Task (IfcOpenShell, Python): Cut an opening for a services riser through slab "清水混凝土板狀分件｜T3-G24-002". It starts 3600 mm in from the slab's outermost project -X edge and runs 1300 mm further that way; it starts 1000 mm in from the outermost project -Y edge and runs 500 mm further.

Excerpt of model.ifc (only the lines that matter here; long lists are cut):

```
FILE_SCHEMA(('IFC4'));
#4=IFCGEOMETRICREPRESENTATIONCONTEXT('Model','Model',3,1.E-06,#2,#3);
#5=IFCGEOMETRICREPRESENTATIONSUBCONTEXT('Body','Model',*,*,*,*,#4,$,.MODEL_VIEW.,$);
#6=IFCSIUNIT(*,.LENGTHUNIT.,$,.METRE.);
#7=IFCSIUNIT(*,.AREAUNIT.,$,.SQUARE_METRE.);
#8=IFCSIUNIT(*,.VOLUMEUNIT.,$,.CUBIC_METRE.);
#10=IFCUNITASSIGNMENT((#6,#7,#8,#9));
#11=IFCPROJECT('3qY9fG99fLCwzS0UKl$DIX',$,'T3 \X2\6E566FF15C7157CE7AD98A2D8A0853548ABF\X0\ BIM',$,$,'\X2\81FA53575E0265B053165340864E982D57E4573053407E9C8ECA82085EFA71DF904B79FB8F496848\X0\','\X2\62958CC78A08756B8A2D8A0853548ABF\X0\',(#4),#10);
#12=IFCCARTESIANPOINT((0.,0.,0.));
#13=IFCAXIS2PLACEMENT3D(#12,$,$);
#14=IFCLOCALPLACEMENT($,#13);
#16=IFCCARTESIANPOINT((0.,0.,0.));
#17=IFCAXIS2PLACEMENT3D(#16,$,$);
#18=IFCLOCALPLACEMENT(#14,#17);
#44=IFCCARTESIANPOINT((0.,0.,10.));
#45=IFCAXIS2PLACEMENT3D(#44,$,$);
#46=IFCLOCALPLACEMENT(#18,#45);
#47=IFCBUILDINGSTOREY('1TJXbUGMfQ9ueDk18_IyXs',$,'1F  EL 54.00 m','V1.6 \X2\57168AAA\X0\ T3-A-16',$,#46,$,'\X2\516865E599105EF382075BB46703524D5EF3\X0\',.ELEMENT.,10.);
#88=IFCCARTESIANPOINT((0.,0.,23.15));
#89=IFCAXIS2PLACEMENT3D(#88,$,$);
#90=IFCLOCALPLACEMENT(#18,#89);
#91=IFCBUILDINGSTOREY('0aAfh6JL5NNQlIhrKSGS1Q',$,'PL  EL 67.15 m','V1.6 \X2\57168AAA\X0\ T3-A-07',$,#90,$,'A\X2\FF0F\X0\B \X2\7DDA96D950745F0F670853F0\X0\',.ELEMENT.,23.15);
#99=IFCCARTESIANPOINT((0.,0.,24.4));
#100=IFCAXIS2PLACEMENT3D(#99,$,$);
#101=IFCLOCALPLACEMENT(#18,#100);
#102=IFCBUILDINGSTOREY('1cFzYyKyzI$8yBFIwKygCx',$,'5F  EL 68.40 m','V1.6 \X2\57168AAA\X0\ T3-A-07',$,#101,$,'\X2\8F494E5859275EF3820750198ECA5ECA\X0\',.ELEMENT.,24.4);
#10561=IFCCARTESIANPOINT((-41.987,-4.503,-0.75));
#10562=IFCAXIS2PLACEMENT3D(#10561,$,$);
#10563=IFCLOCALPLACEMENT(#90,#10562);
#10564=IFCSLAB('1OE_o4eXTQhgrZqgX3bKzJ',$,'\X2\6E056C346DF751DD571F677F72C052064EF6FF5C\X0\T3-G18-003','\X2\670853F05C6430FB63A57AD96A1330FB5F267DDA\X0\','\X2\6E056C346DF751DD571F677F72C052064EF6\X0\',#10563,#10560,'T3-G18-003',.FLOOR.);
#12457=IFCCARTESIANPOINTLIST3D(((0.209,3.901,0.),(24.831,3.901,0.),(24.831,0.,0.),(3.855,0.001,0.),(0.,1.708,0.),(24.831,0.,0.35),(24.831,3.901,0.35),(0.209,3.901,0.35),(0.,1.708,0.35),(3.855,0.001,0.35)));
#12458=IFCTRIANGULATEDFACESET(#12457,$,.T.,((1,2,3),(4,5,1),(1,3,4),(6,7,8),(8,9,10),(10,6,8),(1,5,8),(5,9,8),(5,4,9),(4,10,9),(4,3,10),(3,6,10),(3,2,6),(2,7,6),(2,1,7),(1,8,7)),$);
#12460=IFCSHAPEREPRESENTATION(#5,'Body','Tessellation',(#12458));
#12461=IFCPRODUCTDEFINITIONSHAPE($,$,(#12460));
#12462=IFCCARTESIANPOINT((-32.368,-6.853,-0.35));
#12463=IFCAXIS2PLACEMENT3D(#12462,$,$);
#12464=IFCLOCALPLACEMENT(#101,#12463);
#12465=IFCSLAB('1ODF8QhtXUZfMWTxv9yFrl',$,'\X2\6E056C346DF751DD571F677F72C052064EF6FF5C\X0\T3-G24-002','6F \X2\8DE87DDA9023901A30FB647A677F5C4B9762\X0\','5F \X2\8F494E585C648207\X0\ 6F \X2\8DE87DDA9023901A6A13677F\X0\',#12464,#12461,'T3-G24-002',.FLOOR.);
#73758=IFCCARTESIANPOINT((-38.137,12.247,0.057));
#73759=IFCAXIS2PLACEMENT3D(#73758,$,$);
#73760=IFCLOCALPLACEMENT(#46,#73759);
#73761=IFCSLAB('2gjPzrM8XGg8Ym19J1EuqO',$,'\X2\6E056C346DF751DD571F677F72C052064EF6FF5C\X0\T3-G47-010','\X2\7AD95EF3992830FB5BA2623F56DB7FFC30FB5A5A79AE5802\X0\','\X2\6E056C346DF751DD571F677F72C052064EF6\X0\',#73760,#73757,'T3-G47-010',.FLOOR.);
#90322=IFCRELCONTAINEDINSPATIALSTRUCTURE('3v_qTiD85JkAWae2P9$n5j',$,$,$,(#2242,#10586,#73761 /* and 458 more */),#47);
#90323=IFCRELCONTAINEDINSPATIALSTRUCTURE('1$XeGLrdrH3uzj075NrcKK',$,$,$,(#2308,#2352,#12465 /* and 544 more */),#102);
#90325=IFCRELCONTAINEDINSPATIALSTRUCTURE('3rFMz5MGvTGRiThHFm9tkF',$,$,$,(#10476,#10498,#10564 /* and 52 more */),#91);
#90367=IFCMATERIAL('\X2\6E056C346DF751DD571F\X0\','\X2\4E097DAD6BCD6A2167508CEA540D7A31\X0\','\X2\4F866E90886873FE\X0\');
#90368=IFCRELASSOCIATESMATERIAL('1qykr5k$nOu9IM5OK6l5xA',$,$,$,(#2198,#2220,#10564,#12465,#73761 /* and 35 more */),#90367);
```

```python
import numpy as np
import ifcopenshell
import ifcopenshell.api.feature
import ifcopenshell.api.geometry
import ifcopenshell.api.root
import ifcopenshell.geom
import ifcopenshell.util.placement
import ifcopenshell.util.representation
import ifcopenshell.util.shape
import ifcopenshell.util.unit

model = ifcopenshell.open("model.ifc")
unit_scale = ifcopenshell.util.unit.calculate_unit_scale(model)
settings = ifcopenshell.geom.settings()


def volume(element):
    """Net volume in cubic metres, openings subtracted."""
    shape = ifcopenshell.geom.create_shape(settings, element)
    return ifcopenshell.util.shape.get_volume(shape.geometry)


slab = model.by_id(12465)
before = volume(slab)

# Extent in the slab's own axes, in metres. The edges named are its -X and -Y sides.
slab_shape = ifcopenshell.geom.create_shape(settings, slab)
vertices = ifcopenshell.util.shape.get_vertices(slab_shape.geometry)
x_min, y_min, bottom = vertices.min(axis=0)
top = vertices[:, 2].max()

opening = ifcopenshell.api.root.create_entity(model, ifc_class="IfcOpeningElement", name="Services riser opening", predefined_type="OPENING")
context = ifcopenshell.util.representation.get_context(model, "Model", "Body", "MODEL_VIEW")
width, depth = 1.3, 0.5
outline = [(0.0, 0.0), (width, 0.0), (width, depth), (0.0, depth), (0.0, 0.0)]
# Overshoot both faces by 50 mm so the cut is clean.
shape = ifcopenshell.api.geometry.add_slab_representation(
    model, context=context, depth=top - bottom + 0.1, polyline=outline
)
ifcopenshell.api.geometry.assign_representation(model, product=opening, representation=shape)

matrix = ifcopenshell.util.placement.get_local_placement(slab.ObjectPlacement)
matrix[:, 3] = matrix @ np.append(np.array([x_min + 3.6, y_min + 1, bottom - 0.05]) / unit_scale, 1.0)
ifcopenshell.api.geometry.edit_object_placement(model, product=opening, matrix=matrix, is_si=False)
ifcopenshell.api.feature.add_feature(model, feature=opening, element=slab)

after = volume(slab)

print(f"slab volume {before:.3f} -> {after:.3f} m3")

model.write("model_rev.ifc")
```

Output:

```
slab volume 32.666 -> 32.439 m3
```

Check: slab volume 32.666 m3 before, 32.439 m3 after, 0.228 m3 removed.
